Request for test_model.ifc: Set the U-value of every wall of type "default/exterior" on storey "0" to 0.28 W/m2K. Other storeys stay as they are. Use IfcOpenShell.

First a look at what the model holds.

```python
import ifcopenshell
import ifcopenshell.util.element

model = ifcopenshell.open("test_model.ifc")
print(model.schema)
storey = next(s for s in model.by_type("IfcBuildingStorey") if s.Name == "0")
walls = [e for e in ifcopenshell.util.element.get_decomposition(storey) if e.is_a("IfcWall")]
seen = {}
for e in walls:
    element_type = ifcopenshell.util.element.get_type(e)
    key = (element_type.Name if element_type != e and element_type else None, ifcopenshell.util.element.get_pset(e, "Pset_WallCommon", "ThermalTransmittance"))
    seen[key] = seen.get(key, 0) + 1
for (name, value), count in sorted(seen.items(), key=str):
    print(count, "x", name, "|", value)
```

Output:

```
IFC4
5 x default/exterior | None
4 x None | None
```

```python
import ifcopenshell
import ifcopenshell.api.pset
import ifcopenshell.util.element

model = ifcopenshell.open("test_model.ifc")

storey = next(s for s in model.by_type("IfcBuildingStorey") if s.Name == "0")
walls = [e for e in ifcopenshell.util.element.get_decomposition(storey) if e.is_a("IfcWall")]

count = 0
for e in walls:
    element_type = ifcopenshell.util.element.get_type(e)
    if element_type in (None, e) or element_type.Name != "default/exterior":
        continue
    # add_pset returns the element's existing set when there is one.
    pset = ifcopenshell.api.pset.add_pset(model, product=e, name="Pset_WallCommon")
    ifcopenshell.api.pset.edit_pset(model, pset=pset, properties={"ThermalTransmittance": 0.28})
    count += 1

print(count, "walls updated")

model.write("test_model-out.ifc")
```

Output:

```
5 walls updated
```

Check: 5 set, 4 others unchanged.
